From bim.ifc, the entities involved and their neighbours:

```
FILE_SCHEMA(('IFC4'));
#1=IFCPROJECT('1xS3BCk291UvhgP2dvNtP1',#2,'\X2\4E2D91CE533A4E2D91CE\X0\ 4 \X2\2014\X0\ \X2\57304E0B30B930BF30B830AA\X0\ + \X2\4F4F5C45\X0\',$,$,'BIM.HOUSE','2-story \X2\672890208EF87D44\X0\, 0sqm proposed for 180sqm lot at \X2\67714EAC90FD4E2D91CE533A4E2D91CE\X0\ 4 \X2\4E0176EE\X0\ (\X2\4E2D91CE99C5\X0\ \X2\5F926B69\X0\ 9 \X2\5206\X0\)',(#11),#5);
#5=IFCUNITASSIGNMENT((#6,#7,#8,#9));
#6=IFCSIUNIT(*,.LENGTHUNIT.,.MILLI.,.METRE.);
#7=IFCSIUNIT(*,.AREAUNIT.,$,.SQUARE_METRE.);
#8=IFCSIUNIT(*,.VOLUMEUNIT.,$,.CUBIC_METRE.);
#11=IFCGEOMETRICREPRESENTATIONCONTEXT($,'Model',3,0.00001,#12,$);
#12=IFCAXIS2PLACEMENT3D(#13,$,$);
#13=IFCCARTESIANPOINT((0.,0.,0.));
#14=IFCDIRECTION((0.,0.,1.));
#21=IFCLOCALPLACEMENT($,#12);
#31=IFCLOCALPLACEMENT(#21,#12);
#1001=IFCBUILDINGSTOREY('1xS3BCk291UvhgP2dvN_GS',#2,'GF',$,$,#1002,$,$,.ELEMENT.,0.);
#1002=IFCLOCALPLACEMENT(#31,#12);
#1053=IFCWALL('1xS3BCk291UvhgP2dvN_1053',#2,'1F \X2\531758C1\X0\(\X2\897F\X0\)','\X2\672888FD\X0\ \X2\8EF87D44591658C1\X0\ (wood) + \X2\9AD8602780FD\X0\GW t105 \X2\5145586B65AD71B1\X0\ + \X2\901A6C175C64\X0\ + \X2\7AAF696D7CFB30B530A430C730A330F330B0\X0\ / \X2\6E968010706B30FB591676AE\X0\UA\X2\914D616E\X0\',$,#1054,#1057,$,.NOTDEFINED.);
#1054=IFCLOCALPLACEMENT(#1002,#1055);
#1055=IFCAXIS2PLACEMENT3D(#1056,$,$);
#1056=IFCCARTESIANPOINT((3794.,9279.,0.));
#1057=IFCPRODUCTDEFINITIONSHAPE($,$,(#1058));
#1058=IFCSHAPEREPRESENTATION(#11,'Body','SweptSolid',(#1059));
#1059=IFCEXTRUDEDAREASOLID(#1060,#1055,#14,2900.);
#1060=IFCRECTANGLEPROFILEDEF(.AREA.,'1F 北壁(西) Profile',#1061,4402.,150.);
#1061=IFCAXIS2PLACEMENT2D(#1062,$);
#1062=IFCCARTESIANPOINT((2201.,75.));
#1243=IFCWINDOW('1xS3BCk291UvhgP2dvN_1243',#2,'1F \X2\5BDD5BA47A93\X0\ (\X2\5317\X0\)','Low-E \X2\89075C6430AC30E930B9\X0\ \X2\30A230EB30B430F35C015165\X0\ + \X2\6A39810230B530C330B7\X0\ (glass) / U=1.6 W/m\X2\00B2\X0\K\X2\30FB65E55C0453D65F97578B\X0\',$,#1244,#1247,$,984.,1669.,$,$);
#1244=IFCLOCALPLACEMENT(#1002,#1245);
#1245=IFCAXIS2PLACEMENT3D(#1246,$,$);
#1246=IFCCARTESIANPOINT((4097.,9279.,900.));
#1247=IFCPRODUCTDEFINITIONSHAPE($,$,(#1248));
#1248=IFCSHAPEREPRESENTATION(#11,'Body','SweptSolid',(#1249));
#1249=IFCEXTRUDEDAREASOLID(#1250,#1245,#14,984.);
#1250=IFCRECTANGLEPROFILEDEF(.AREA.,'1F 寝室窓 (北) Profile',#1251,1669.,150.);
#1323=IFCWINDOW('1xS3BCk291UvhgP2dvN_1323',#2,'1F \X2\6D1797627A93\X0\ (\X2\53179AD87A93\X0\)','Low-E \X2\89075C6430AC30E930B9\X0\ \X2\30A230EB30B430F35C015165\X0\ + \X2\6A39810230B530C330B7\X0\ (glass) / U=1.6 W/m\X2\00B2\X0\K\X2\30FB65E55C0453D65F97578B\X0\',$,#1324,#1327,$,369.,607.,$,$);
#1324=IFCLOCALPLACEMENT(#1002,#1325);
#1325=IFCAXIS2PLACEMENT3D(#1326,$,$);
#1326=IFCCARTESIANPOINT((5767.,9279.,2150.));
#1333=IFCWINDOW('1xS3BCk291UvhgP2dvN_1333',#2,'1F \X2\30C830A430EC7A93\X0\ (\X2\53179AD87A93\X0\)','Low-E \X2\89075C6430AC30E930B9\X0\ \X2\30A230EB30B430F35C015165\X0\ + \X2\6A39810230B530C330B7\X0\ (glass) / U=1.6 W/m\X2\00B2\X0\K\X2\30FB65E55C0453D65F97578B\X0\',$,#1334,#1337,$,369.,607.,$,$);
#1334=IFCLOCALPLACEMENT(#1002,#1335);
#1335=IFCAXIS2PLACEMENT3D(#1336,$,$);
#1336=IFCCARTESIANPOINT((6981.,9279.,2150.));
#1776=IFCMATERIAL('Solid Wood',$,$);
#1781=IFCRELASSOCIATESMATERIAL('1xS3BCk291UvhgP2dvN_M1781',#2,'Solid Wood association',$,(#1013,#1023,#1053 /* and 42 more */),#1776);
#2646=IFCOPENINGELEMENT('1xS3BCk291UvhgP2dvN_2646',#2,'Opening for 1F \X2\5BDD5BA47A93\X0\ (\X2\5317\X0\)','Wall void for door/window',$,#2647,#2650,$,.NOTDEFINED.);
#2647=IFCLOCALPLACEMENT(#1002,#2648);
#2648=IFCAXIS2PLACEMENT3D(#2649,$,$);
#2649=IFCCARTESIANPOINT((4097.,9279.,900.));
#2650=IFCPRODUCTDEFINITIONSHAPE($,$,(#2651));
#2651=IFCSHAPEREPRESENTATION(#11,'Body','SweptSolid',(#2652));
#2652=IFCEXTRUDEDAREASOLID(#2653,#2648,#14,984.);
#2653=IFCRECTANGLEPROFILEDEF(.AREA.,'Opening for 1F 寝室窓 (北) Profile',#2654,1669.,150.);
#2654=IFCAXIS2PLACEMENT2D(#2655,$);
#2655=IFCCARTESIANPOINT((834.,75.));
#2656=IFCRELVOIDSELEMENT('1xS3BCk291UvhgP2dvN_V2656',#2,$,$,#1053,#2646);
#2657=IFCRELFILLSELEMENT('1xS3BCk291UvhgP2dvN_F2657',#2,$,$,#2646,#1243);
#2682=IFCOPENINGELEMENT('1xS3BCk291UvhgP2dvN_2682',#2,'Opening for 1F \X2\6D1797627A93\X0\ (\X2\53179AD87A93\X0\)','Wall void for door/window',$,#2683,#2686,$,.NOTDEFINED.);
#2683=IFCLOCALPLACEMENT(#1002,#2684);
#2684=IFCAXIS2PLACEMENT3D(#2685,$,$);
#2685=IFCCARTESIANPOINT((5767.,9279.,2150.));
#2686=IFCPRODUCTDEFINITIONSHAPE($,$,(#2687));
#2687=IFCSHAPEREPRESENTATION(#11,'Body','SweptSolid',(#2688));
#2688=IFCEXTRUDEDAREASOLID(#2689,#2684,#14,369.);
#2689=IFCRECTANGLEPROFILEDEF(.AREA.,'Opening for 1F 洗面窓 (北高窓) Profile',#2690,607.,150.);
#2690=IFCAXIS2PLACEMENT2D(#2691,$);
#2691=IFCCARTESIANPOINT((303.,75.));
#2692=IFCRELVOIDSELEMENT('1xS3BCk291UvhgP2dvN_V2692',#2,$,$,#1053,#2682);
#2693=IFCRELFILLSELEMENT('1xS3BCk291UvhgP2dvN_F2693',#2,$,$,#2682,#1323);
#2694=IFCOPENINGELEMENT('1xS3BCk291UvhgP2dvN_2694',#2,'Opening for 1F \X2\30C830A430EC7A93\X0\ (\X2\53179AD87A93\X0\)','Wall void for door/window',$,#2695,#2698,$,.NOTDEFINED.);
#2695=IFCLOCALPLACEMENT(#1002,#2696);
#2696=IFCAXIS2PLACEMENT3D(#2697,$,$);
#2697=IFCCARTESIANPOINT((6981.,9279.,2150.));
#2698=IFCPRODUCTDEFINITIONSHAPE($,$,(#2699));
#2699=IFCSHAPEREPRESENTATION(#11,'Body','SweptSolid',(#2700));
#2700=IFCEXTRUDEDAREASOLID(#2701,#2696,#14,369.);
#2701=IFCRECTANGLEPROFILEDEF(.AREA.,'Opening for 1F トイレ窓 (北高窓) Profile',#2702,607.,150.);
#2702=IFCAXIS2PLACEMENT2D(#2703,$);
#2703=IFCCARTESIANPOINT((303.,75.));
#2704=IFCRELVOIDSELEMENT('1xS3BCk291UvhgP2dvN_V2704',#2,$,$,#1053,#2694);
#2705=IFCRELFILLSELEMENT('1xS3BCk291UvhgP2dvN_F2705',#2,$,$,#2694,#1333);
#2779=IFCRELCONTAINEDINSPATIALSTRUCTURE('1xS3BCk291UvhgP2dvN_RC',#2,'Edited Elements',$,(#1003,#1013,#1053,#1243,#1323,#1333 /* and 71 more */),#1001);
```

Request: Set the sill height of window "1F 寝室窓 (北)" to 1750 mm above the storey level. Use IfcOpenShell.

```python
import numpy as np
import ifcopenshell
import ifcopenshell.api.geometry
import ifcopenshell.geom
import ifcopenshell.util.element
import ifcopenshell.util.placement
import ifcopenshell.util.shape
import ifcopenshell.util.unit

model = ifcopenshell.open("bim.ifc")
unit_scale = ifcopenshell.util.unit.calculate_unit_scale(model)

window = model.by_guid("1xS3BCk291UvhgP2dvN_1243")
opening = window.FillsVoids[0].RelatingOpeningElement
storey = ifcopenshell.util.element.get_container(window, ifc_class="IfcBuildingStorey")
level = ifcopenshell.util.placement.get_local_placement(storey.ObjectPlacement)[2, 3]

# The opening's origin need not be at the sill, so measure its lowest point.
shape = ifcopenshell.geom.create_shape(ifcopenshell.geom.settings(), opening)
bottom = ifcopenshell.util.shape.get_shape_bottom_elevation(shape, shape.geometry) / unit_scale
dz = level + 1750.0 - bottom

shift = np.array([0.0, 0.0, dz])
# The window is not placed relative to its opening, so move both.
for product in (opening, window):
    matrix = ifcopenshell.util.placement.get_local_placement(product.ObjectPlacement)
    matrix[:3, 3] += shift
    ifcopenshell.api.geometry.edit_object_placement(model, product=product, matrix=matrix, is_si=False)

print(f"moved by {dz * unit_scale:+.3f} m")

model.write("bim-out.ifc")
```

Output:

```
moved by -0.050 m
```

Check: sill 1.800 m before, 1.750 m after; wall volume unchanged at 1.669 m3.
